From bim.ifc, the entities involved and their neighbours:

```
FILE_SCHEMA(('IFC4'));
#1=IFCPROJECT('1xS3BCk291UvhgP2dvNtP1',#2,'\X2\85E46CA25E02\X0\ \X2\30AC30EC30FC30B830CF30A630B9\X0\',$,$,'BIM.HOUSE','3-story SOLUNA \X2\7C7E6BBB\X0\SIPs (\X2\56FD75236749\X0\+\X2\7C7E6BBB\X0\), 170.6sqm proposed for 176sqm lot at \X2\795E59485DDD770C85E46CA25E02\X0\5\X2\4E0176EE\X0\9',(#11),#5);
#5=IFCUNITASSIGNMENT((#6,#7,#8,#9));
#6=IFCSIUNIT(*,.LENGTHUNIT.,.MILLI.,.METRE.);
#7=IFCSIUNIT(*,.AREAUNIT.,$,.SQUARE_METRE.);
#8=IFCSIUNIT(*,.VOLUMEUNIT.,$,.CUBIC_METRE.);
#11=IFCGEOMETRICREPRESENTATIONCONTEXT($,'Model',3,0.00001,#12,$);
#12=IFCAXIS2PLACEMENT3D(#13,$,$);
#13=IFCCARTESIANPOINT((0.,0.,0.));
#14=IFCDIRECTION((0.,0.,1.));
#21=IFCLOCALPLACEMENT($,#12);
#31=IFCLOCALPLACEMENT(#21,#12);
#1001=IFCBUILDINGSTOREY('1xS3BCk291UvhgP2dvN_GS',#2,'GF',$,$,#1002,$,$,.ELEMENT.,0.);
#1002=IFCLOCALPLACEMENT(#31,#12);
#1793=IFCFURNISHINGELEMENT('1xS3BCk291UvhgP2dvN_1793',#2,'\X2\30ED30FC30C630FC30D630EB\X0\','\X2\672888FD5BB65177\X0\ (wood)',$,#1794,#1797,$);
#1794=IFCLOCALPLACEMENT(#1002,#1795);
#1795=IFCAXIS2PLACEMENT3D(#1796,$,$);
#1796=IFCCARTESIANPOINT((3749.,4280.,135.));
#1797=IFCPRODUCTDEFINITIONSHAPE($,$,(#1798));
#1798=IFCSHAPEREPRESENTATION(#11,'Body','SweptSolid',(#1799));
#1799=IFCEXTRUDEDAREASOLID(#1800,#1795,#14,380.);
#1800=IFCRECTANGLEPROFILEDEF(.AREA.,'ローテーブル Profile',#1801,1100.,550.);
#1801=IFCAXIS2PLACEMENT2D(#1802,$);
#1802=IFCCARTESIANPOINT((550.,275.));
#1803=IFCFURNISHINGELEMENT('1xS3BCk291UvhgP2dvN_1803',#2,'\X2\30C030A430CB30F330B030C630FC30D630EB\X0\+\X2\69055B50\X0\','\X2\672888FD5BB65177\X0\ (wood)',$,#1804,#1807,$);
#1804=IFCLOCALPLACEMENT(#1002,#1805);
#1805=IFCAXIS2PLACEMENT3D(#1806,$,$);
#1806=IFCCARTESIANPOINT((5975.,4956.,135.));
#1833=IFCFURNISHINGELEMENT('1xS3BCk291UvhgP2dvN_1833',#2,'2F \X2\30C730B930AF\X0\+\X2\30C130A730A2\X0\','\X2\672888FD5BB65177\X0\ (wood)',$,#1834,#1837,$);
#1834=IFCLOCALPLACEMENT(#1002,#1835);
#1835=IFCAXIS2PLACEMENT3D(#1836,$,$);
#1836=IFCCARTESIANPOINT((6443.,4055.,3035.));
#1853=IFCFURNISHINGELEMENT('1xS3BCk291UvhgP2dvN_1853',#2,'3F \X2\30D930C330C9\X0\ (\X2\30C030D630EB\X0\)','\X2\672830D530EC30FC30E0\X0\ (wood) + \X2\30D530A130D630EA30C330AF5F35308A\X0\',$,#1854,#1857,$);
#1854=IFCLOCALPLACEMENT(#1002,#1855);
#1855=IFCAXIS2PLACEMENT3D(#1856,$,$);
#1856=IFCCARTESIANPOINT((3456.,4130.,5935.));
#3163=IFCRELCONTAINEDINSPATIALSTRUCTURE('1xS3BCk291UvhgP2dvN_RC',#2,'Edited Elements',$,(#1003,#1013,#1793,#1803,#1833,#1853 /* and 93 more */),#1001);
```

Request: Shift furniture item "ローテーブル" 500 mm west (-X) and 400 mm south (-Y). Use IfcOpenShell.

```python
import ifcopenshell
import ifcopenshell.api.geometry
import ifcopenshell.util.placement
import ifcopenshell.util.unit

model = ifcopenshell.open("bim.ifc")
unit_scale = ifcopenshell.util.unit.calculate_unit_scale(model)

item = model.by_guid("1xS3BCk291UvhgP2dvN_1793")
matrix = ifcopenshell.util.placement.get_local_placement(item.ObjectPlacement)
matrix[0, 3] -= 0.5 / unit_scale
matrix[1, 3] -= 0.4 / unit_scale
ifcopenshell.api.geometry.edit_object_placement(model, product=item, matrix=matrix, is_si=False)

print(ifcopenshell.util.placement.get_local_placement(item.ObjectPlacement).round(3) + 0.0)

model.write("bim_edited.ifc")
```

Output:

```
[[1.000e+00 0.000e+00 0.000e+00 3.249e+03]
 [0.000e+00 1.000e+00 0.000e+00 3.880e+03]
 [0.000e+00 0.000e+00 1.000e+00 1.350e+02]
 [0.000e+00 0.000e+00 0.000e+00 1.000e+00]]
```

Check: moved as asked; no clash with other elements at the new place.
